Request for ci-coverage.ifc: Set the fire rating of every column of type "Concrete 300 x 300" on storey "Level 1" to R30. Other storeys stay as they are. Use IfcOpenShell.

First a look at what the model holds.

```python
import ifcopenshell
import ifcopenshell.util.element

model = ifcopenshell.open("ci-coverage.ifc")
print(model.schema)
storey = next(s for s in model.by_type("IfcBuildingStorey") if s.Name == "Level 1")
columns = [e for e in ifcopenshell.util.element.get_decomposition(storey) if e.is_a("IfcColumn")]
seen = {}
for e in columns:
    element_type = ifcopenshell.util.element.get_type(e)
    key = (element_type.Name if element_type != e and element_type else None, ifcopenshell.util.element.get_pset(e, "Pset_ColumnCommon", "FireRating"))
    seen[key] = seen.get(key, 0) + 1
for (name, value), count in sorted(seen.items(), key=str):
    print(count, "x", name, "|", value)
```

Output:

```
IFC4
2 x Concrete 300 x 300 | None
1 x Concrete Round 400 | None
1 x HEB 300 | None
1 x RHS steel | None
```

```python
import ifcopenshell
import ifcopenshell.api.pset
import ifcopenshell.util.element

model = ifcopenshell.open("ci-coverage.ifc")

storey = next(s for s in model.by_type("IfcBuildingStorey") if s.Name == "Level 1")
columns = [e for e in ifcopenshell.util.element.get_decomposition(storey) if e.is_a("IfcColumn")]

count = 0
for e in columns:
    element_type = ifcopenshell.util.element.get_type(e)
    if element_type in (None, e) or element_type.Name != "Concrete 300 x 300":
        continue
    # add_pset returns the element's existing set when there is one.
    pset = ifcopenshell.api.pset.add_pset(model, product=e, name="Pset_ColumnCommon")
    ifcopenshell.api.pset.edit_pset(model, pset=pset, properties={"FireRating": "R30"})
    count += 1

print(count, "columns updated")

model.write("ci-coverage_edited.ifc")
```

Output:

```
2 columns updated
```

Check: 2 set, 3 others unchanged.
